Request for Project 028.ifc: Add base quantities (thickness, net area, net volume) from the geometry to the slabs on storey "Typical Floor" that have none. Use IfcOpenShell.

First a look at what the model holds.

```python
import ifcopenshell
import ifcopenshell.util.element
import ifcopenshell.util.unit

model = ifcopenshell.open("Project 028.ifc")
print(model.schema)
for unit_type in ("LENGTHUNIT", "AREAUNIT", "VOLUMEUNIT"):
    print(unit_type, ifcopenshell.util.unit.calculate_unit_scale(model, unit_type))
storey = next(s for s in model.by_type("IfcBuildingStorey") if s.Name == "Typical Floor")
slabs = [e for e in ifcopenshell.util.element.get_decomposition(storey) if e.is_a("IfcSlab")]
for e in sorted(slabs, key=lambda e: e.id()):
    print(e.id(), e.is_a(), e.Name, list(ifcopenshell.util.element.get_psets(e, qtos_only=True)), sep=" | ")
```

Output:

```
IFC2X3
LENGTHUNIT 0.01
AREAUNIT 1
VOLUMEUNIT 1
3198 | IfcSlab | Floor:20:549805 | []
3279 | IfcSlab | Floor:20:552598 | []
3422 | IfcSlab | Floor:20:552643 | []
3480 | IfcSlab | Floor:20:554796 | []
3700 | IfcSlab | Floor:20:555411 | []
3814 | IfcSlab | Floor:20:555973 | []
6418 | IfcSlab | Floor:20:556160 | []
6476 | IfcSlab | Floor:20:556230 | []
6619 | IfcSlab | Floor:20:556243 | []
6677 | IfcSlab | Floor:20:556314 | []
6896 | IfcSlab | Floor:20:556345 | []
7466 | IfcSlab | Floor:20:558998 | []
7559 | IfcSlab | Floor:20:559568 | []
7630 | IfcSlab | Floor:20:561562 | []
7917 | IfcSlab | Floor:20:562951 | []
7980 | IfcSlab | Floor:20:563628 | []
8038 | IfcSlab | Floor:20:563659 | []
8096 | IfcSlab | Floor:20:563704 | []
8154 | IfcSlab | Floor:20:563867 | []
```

```python
import ifcopenshell
import ifcopenshell.api.pset
import ifcopenshell.geom
import ifcopenshell.util.element
import ifcopenshell.util.shape
import ifcopenshell.util.unit

model = ifcopenshell.open("Project 028.ifc")
unit_scale = ifcopenshell.util.unit.calculate_unit_scale(model)
area_scale = ifcopenshell.util.unit.calculate_unit_scale(model, "AREAUNIT")
volume_scale = ifcopenshell.util.unit.calculate_unit_scale(model, "VOLUMEUNIT")
settings = ifcopenshell.geom.settings()

storey = next(s for s in model.by_type("IfcBuildingStorey") if s.Name == "Typical Floor")
slabs = [e for e in ifcopenshell.util.element.get_decomposition(storey) if e.is_a("IfcSlab")]

for e in sorted(slabs, key=lambda e: e.id()):
    if ifcopenshell.util.element.get_psets(e, qtos_only=True, should_inherit=False):
        continue
    # Geometry comes back in metres, in the element's own axes.
    shape = ifcopenshell.geom.create_shape(settings, e)
    values = {
        "Width": ifcopenshell.util.shape.get_z(shape.geometry) / unit_scale,
        "NetArea": ifcopenshell.util.shape.get_footprint_area(shape.geometry) / area_scale,
        "NetVolume": ifcopenshell.util.shape.get_volume(shape.geometry) / volume_scale,
    }
    qto = ifcopenshell.api.pset.add_qto(model, product=e, name="BaseQuantities")
    ifcopenshell.api.pset.edit_qto(model, qto=qto, properties=values)
    print(e.id(), {k: round(v, 3) for k, v in values.items()})

model.write("Project 028_v2.ifc")
```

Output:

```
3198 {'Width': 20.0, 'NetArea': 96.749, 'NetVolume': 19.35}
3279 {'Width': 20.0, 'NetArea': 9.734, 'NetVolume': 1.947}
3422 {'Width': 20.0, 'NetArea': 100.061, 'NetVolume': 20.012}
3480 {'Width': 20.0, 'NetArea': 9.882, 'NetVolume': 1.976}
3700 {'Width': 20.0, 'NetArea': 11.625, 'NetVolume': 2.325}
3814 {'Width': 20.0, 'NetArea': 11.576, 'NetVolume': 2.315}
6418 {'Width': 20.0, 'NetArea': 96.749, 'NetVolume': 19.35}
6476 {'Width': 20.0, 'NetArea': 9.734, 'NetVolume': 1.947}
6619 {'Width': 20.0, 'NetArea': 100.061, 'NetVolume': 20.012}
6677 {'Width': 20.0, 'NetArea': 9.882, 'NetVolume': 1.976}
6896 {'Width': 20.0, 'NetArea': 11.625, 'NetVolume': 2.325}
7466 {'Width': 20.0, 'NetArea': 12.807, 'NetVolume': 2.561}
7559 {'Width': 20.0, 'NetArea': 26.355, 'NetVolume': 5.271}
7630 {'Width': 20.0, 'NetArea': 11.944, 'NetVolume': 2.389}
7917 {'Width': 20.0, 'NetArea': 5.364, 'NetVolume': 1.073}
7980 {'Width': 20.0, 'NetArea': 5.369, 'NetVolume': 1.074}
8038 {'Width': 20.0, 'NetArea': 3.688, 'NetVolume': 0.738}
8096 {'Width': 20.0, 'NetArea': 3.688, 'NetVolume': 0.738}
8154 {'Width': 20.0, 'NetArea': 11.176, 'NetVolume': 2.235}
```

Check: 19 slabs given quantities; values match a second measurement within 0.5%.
